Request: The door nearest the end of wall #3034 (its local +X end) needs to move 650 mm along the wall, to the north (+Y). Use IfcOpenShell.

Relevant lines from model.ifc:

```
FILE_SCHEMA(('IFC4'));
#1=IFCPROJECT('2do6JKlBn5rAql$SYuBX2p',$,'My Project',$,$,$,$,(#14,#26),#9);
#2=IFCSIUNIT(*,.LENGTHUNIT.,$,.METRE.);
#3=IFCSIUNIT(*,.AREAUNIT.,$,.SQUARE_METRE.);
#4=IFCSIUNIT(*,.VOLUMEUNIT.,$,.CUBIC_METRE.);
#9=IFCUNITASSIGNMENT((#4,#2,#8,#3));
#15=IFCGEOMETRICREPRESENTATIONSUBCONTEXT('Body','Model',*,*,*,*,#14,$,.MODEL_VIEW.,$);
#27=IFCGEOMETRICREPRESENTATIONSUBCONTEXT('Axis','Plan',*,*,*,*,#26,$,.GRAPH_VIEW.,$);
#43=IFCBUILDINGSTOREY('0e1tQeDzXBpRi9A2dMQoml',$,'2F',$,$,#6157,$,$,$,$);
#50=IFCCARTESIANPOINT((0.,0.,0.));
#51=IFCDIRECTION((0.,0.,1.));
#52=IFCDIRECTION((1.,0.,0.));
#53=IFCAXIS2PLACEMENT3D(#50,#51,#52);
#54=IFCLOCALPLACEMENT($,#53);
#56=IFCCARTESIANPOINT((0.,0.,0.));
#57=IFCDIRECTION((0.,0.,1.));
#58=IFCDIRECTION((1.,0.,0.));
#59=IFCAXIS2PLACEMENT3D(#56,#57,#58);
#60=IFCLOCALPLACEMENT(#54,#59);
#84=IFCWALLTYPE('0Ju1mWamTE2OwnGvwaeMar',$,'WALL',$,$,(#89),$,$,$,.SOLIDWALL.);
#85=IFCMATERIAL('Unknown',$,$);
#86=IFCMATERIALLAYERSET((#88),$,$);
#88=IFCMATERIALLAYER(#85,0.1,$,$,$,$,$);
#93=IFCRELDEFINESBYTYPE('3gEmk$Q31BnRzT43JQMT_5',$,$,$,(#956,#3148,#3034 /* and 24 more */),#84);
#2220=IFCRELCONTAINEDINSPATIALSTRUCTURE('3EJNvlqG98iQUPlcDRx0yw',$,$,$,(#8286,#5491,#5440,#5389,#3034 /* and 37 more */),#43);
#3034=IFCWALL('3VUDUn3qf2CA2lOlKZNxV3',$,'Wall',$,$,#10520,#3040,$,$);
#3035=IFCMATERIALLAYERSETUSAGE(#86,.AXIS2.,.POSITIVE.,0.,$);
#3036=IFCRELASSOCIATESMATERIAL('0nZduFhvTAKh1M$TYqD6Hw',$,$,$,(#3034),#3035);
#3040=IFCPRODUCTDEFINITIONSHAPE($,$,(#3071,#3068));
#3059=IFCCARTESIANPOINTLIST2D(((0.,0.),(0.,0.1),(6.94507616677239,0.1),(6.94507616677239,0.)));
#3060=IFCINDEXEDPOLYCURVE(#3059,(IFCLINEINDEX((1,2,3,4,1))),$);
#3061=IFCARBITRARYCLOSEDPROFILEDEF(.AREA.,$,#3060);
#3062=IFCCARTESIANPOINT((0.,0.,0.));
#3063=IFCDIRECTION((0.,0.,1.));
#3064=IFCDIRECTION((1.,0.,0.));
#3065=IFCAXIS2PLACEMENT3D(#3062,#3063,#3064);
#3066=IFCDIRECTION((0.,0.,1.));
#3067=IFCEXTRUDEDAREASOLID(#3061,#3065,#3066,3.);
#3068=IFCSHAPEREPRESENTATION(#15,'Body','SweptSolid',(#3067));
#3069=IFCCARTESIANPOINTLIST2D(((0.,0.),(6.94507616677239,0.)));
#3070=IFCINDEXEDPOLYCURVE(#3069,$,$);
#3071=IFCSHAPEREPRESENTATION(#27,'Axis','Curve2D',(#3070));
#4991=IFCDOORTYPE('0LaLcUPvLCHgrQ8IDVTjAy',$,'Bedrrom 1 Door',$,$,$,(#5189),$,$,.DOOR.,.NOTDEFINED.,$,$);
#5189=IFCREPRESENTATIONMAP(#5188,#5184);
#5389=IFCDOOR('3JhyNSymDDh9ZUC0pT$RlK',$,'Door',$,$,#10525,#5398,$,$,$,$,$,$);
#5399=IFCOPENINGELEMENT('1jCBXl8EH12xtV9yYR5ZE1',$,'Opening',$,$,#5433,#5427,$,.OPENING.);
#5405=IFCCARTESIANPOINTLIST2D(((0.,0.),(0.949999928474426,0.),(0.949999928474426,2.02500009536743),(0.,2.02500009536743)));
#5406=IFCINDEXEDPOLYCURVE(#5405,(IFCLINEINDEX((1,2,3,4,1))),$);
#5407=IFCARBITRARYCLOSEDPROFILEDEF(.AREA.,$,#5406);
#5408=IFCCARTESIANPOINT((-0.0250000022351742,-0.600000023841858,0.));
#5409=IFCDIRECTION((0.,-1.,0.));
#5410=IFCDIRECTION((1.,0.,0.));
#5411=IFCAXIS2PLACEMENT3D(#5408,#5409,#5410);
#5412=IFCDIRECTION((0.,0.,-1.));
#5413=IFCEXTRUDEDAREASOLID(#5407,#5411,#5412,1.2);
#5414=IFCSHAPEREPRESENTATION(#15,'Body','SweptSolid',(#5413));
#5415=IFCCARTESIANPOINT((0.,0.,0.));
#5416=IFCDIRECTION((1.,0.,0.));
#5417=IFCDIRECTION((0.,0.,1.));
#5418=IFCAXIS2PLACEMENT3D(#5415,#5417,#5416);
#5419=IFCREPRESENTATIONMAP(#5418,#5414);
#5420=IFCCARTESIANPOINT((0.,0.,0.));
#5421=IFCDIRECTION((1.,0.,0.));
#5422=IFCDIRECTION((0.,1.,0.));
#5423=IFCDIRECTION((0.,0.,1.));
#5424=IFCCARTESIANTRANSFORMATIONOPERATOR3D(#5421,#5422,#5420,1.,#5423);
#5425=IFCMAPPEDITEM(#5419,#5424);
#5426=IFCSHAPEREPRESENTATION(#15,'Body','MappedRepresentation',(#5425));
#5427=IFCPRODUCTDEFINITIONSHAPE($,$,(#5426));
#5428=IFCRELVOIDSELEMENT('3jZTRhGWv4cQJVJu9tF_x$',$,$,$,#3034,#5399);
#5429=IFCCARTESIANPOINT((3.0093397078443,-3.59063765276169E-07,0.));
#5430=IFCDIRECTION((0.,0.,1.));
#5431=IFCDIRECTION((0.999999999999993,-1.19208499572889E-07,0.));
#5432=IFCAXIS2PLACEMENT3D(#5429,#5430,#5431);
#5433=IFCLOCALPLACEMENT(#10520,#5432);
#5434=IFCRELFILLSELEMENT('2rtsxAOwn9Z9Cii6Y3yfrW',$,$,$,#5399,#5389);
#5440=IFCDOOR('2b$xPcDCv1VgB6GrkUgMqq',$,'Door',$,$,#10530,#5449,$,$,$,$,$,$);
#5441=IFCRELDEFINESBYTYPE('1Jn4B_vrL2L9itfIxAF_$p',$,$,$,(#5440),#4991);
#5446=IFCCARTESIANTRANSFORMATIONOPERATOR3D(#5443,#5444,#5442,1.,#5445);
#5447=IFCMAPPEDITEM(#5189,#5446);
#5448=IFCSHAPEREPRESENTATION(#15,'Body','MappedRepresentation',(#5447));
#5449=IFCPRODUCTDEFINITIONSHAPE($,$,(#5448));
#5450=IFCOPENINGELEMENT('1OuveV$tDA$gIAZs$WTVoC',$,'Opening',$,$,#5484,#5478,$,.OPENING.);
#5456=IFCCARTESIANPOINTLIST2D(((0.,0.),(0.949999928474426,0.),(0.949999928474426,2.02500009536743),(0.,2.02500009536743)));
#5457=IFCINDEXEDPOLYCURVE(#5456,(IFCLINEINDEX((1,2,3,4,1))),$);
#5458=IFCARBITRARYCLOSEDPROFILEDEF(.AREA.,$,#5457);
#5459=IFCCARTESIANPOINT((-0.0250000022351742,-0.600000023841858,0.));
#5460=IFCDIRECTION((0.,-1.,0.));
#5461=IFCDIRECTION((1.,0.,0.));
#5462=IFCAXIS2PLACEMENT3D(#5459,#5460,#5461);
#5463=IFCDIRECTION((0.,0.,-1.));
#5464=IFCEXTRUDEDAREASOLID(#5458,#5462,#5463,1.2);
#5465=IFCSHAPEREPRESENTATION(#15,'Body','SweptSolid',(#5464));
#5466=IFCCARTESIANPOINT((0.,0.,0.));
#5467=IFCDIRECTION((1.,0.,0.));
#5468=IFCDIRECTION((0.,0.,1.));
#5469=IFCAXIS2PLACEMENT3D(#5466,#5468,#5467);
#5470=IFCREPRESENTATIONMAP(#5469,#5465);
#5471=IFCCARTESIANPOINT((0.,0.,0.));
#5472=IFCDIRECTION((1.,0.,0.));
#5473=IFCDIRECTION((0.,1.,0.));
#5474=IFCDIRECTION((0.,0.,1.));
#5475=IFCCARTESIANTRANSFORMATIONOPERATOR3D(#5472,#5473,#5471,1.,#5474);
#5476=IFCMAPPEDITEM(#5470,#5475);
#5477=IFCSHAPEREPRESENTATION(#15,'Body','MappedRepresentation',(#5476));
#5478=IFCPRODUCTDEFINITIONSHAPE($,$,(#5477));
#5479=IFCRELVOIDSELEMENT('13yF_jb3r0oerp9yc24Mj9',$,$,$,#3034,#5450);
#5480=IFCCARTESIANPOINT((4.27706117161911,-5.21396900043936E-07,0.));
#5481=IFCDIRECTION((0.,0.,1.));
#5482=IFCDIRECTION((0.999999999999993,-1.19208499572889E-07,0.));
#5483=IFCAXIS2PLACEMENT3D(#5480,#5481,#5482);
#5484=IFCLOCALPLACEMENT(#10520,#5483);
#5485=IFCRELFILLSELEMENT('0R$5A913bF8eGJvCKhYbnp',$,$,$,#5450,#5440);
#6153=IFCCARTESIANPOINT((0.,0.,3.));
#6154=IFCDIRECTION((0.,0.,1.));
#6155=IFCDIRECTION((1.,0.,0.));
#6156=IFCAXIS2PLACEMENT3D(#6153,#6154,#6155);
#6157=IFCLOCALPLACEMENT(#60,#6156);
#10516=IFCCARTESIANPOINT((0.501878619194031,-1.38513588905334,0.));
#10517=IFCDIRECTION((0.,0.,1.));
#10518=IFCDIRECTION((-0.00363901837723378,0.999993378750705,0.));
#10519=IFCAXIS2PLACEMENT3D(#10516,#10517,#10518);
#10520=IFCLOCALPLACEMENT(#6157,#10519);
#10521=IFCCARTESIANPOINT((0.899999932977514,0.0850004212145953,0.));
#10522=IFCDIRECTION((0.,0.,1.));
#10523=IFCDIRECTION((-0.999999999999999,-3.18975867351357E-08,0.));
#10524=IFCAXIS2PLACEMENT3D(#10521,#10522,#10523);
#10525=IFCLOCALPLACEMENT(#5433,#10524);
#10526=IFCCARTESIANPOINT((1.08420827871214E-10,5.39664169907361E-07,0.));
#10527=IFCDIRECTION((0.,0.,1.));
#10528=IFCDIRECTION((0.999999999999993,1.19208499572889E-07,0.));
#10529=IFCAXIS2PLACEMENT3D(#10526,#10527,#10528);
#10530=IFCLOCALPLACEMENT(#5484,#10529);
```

```python
import ifcopenshell
import ifcopenshell.api.geometry
import ifcopenshell.util.placement

model = ifcopenshell.open("model.ifc")

door = model.by_guid("2b$xPcDCv1VgB6GrkUgMqq")
opening = door.FillsVoids[0].RelatingOpeningElement
wall = opening.VoidsElements[0].RelatingBuildingElement

wall_matrix = ifcopenshell.util.placement.get_local_placement(wall.ObjectPlacement)
shift = wall_matrix[:3, 0] * 0.65
before = ifcopenshell.util.placement.get_local_placement(door.ObjectPlacement)[:3, 3].copy()

# The door is placed relative to its opening, so it follows when the opening moves.
matrix = ifcopenshell.util.placement.get_local_placement(opening.ObjectPlacement)
matrix[:3, 3] += shift
ifcopenshell.api.geometry.edit_object_placement(
    model, product=opening, matrix=matrix, is_si=False, should_transform_children=True
)

after = ifcopenshell.util.placement.get_local_placement(door.ObjectPlacement)[:3, 3]
print("door moved by", (after - before).round(3) + 0.0)

model.write("model_edited.ifc")
```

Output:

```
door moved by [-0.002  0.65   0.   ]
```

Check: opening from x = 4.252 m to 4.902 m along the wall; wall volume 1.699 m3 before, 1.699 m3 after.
